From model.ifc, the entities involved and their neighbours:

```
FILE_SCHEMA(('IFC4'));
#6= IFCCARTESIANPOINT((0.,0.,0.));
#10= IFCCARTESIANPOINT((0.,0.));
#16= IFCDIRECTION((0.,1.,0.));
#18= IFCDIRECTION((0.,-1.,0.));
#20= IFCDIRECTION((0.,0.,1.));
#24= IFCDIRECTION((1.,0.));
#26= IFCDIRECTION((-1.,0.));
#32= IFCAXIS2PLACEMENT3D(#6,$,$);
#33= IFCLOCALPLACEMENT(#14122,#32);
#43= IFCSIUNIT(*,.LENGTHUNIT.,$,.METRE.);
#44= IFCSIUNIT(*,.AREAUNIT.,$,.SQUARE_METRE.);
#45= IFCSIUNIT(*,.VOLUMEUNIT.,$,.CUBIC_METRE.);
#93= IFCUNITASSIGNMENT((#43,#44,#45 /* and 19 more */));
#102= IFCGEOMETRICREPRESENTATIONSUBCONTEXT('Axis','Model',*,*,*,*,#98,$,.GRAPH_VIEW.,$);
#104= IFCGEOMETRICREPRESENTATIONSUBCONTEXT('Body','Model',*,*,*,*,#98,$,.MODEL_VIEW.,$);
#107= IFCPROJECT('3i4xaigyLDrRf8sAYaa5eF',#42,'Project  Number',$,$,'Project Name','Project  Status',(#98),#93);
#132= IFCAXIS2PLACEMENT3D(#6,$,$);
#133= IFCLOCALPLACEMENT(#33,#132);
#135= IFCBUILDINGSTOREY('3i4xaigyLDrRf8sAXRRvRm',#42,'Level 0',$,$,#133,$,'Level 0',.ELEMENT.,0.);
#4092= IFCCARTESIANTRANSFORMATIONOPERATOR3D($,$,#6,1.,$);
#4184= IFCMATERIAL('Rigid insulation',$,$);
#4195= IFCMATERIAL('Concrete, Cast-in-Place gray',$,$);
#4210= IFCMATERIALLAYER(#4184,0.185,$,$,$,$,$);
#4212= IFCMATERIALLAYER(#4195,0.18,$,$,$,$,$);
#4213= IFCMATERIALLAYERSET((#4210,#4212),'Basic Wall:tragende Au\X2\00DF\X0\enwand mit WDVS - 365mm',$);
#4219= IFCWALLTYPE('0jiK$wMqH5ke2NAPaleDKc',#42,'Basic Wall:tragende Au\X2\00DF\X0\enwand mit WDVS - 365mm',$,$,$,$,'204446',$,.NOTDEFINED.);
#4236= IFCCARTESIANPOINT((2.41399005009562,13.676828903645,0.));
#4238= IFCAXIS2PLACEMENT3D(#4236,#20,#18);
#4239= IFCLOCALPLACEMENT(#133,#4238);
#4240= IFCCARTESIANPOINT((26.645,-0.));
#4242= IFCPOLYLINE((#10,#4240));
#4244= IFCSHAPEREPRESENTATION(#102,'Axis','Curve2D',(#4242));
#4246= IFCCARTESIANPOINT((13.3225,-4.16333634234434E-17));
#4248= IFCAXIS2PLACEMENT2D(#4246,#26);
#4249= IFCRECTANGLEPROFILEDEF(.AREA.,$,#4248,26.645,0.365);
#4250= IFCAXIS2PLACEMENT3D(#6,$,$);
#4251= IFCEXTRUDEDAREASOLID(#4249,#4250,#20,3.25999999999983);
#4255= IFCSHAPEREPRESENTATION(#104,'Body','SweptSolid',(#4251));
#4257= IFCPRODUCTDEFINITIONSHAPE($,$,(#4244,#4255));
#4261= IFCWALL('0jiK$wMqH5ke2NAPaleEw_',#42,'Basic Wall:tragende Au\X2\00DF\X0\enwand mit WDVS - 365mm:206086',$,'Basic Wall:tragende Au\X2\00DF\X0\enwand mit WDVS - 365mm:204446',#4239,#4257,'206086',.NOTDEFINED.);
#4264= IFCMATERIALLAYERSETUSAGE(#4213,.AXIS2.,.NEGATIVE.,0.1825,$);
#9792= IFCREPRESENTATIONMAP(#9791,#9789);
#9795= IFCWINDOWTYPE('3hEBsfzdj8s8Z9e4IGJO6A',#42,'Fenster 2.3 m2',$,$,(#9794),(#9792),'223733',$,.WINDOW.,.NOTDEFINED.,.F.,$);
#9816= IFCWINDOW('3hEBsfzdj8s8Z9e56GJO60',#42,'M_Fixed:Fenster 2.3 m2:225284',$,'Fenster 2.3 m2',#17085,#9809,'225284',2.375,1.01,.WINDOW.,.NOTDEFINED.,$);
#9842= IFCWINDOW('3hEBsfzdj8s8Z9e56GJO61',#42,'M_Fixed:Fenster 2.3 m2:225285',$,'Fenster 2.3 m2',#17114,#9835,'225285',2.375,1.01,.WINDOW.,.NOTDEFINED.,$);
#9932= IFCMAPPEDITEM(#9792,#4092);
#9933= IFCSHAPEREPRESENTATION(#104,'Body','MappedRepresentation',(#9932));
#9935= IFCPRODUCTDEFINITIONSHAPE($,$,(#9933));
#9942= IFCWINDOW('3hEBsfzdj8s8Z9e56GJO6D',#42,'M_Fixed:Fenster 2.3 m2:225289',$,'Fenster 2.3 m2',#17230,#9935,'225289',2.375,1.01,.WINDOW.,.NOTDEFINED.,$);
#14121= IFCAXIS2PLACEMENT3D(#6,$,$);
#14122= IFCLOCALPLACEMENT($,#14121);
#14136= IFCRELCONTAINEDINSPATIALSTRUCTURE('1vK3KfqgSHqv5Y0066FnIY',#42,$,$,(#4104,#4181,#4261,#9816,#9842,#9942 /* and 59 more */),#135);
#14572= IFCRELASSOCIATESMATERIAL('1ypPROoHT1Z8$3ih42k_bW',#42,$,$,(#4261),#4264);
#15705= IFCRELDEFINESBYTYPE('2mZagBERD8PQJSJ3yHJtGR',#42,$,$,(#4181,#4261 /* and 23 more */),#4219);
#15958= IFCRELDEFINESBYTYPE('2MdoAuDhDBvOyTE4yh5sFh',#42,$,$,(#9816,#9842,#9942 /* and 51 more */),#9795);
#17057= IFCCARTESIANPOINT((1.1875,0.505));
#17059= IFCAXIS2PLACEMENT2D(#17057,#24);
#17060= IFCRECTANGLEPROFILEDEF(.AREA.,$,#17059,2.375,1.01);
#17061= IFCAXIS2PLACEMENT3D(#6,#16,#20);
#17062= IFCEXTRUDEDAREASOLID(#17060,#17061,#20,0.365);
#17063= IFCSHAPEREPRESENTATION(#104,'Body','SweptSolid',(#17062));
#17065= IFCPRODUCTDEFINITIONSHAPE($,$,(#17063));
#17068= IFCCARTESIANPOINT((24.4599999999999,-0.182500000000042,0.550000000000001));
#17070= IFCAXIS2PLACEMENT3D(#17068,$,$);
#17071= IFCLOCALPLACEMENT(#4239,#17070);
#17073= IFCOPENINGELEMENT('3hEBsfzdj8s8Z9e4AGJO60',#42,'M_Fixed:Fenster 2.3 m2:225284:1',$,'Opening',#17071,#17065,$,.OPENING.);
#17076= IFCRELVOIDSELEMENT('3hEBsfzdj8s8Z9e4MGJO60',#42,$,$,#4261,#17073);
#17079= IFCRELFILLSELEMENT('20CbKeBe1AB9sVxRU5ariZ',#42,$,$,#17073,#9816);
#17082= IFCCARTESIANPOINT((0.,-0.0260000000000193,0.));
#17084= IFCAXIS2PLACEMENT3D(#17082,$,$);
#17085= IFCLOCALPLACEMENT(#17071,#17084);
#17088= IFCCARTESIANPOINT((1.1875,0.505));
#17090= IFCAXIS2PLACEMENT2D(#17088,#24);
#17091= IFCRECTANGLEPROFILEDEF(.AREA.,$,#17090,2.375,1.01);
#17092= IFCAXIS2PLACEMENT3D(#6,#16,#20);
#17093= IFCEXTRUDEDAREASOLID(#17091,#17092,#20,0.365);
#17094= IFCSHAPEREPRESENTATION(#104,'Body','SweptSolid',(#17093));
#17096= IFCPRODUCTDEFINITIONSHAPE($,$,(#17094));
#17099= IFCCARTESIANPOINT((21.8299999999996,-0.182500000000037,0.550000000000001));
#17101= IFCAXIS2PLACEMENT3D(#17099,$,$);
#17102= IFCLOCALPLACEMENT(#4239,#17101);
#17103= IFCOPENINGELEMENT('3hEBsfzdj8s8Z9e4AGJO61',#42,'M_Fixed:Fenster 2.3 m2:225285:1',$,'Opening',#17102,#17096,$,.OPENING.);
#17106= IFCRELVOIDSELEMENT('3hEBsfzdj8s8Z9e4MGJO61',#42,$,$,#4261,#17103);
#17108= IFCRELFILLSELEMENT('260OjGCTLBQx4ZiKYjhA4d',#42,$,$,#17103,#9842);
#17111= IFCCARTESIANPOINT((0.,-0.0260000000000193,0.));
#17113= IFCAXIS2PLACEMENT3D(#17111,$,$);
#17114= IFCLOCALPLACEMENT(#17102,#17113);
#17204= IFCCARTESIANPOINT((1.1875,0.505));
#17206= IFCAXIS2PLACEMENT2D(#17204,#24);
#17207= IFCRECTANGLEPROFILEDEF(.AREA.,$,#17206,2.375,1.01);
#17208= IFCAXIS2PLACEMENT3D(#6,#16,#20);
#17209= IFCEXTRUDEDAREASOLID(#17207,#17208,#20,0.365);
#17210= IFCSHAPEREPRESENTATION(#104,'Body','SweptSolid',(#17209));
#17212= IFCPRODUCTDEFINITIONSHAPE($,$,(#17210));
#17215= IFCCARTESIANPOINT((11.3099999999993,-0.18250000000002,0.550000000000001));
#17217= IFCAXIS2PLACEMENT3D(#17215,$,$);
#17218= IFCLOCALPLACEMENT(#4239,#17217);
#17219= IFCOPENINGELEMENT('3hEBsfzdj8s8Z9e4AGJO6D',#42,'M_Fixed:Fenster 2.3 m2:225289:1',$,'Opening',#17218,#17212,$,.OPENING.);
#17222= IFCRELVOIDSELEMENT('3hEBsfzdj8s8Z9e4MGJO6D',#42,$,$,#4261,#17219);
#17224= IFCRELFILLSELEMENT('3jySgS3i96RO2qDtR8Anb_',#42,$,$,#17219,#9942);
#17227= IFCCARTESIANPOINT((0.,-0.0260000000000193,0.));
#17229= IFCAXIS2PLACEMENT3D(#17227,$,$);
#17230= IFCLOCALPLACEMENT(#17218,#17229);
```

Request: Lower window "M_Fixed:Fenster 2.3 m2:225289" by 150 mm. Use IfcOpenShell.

```python
import numpy as np
import ifcopenshell
import ifcopenshell.api.geometry
import ifcopenshell.util.placement
import ifcopenshell.util.unit

model = ifcopenshell.open("model.ifc")
unit_scale = ifcopenshell.util.unit.calculate_unit_scale(model)

window = model.by_guid("3hEBsfzdj8s8Z9e56GJO6D")
opening = window.FillsVoids[0].RelatingOpeningElement
dz = -0.15

shift = np.array([0.0, 0.0, dz])
# The window is placed relative to its opening, so it follows when the opening moves.
matrix = ifcopenshell.util.placement.get_local_placement(opening.ObjectPlacement)
matrix[:3, 3] += shift
ifcopenshell.api.geometry.edit_object_placement(
    model, product=opening, matrix=matrix, is_si=False, should_transform_children=True
)

print(f"moved by {dz * unit_scale:+.3f} m")

model.write("model_updated.ifc")
```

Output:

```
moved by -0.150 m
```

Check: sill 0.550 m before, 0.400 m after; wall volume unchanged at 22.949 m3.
